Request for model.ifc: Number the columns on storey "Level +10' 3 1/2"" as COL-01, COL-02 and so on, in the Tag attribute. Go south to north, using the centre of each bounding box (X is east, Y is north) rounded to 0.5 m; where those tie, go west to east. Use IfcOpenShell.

First a look at what the model holds.

```python
import ifcopenshell
import ifcopenshell.util.element
import ifcopenshell.util.placement

model = ifcopenshell.open("model.ifc")
print(model.schema)
storey = next(s for s in model.by_type("IfcBuildingStorey") if s.Name == 'Level +10\' 3 1/2"')
columns = [e for e in ifcopenshell.util.element.get_decomposition(storey) if e.is_a("IfcColumn")]
for e in sorted(columns, key=lambda e: e.id()):
    origin = ifcopenshell.util.placement.get_local_placement(e.ObjectPlacement)[:3, 3]
    print(e.id(), e.Tag, e.Name, origin.round(2) + 0.0, sep=" | ")
```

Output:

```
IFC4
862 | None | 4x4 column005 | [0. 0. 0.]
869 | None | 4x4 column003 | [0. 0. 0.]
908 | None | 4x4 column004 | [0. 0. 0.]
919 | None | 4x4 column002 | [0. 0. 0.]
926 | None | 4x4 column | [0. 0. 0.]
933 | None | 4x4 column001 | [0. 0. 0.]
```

```python
import ifcopenshell
import ifcopenshell.geom
import ifcopenshell.util.element
import ifcopenshell.util.shape

model = ifcopenshell.open("model.ifc")
settings = ifcopenshell.geom.settings()
settings.set("use-world-coords", True)


def centre(element):
    shape = ifcopenshell.geom.create_shape(settings, element)
    return ifcopenshell.util.shape.get_bbox_centroid(shape.geometry)


storey = next(s for s in model.by_type("IfcBuildingStorey") if s.Name == 'Level +10\' 3 1/2"')
columns = [e for e in ifcopenshell.util.element.get_decomposition(storey) if e.is_a("IfcColumn")]

# Insertion points can sit at a corner or the storey origin, so sort by the geometry (in metres).
centres = {e: centre(e) for e in columns}
columns.sort(key=lambda e: (round(centres[e][1] / 0.5), centres[e][0]))

for i, e in enumerate(columns, start=1):
    number = f"COL-{i:02d}"
    e.Tag = number
    print(e.id(), number)

model.write("model_edited.ifc")
```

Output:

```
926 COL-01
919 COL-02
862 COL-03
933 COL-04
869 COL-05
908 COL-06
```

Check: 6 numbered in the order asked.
